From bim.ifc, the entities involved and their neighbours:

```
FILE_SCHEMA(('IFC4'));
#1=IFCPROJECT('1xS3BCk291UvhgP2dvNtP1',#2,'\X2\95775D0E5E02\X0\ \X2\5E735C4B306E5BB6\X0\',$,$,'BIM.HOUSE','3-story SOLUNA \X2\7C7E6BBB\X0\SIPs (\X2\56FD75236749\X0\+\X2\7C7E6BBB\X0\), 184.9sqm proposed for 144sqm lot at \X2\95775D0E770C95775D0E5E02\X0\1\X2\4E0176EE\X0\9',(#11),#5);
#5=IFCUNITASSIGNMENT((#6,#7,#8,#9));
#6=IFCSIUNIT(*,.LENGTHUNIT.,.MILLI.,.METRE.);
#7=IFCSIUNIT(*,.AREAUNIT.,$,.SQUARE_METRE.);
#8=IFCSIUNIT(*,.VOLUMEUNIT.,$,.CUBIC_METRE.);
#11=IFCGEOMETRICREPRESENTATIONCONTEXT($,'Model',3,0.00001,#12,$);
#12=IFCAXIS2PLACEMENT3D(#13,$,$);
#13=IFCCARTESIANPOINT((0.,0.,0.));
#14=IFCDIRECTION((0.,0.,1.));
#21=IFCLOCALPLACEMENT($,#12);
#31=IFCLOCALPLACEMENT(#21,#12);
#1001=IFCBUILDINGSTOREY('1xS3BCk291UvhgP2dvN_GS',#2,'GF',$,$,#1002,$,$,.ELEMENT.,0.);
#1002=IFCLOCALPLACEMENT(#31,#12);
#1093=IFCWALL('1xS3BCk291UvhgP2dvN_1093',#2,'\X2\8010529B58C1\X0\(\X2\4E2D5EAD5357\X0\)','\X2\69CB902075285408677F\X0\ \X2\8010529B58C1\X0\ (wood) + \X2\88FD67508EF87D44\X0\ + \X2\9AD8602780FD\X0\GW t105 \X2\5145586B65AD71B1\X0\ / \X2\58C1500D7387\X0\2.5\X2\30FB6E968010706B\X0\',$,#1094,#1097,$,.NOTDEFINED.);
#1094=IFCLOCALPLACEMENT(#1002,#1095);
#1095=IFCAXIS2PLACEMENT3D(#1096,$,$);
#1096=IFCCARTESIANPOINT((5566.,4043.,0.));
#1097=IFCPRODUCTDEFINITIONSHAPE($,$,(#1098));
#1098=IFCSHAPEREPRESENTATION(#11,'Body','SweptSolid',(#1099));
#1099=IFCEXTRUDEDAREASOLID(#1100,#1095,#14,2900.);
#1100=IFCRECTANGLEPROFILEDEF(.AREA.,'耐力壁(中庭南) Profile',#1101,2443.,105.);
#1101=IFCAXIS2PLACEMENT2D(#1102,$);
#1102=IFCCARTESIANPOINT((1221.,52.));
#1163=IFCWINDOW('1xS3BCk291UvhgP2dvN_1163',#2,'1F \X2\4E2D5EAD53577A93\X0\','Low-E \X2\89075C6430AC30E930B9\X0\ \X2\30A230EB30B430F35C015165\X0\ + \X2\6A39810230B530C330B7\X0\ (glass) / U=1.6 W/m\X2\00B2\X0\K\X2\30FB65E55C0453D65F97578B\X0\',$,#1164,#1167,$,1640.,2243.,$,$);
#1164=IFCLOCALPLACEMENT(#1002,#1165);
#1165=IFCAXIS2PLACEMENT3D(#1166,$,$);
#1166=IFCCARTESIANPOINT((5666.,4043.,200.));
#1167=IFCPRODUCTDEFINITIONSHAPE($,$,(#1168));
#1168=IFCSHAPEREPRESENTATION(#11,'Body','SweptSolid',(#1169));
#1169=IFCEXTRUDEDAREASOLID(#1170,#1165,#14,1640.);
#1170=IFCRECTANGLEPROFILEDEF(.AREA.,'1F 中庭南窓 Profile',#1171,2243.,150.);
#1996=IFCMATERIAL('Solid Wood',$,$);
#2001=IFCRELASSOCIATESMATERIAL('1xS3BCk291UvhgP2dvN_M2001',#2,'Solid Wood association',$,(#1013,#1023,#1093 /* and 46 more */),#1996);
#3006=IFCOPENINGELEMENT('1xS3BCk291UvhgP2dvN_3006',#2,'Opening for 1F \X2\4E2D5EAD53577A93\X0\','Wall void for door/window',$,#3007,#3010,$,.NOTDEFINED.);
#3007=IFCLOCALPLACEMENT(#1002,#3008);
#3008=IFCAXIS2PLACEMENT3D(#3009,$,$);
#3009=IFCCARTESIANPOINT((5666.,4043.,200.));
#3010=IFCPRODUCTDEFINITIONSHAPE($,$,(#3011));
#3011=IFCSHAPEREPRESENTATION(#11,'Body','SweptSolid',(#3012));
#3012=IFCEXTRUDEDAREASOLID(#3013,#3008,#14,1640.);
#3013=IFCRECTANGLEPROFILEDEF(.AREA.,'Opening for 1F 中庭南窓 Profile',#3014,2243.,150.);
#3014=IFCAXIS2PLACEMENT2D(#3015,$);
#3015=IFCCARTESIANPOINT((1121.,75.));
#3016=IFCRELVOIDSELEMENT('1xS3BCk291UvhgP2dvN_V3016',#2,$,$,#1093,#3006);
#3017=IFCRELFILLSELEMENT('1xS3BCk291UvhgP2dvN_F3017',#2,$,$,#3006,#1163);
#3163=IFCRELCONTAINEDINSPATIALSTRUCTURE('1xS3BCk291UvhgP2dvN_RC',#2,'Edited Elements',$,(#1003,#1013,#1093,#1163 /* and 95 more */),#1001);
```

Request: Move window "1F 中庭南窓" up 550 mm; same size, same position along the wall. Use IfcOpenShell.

```python
import numpy as np
import ifcopenshell
import ifcopenshell.api.geometry
import ifcopenshell.util.placement
import ifcopenshell.util.unit

model = ifcopenshell.open("bim.ifc")
unit_scale = ifcopenshell.util.unit.calculate_unit_scale(model)

window = model.by_id(1163)
opening = window.FillsVoids[0].RelatingOpeningElement
dz = 0.55 / unit_scale

shift = np.array([0.0, 0.0, dz])
# The window is not placed relative to its opening, so move both.
for product in (opening, window):
    matrix = ifcopenshell.util.placement.get_local_placement(product.ObjectPlacement)
    matrix[:3, 3] += shift
    ifcopenshell.api.geometry.edit_object_placement(model, product=product, matrix=matrix, is_si=False)

print(f"moved by {dz * unit_scale:+.3f} m")

model.write("bim-out.ifc")
```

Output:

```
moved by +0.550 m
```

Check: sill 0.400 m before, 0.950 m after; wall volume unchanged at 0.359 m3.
